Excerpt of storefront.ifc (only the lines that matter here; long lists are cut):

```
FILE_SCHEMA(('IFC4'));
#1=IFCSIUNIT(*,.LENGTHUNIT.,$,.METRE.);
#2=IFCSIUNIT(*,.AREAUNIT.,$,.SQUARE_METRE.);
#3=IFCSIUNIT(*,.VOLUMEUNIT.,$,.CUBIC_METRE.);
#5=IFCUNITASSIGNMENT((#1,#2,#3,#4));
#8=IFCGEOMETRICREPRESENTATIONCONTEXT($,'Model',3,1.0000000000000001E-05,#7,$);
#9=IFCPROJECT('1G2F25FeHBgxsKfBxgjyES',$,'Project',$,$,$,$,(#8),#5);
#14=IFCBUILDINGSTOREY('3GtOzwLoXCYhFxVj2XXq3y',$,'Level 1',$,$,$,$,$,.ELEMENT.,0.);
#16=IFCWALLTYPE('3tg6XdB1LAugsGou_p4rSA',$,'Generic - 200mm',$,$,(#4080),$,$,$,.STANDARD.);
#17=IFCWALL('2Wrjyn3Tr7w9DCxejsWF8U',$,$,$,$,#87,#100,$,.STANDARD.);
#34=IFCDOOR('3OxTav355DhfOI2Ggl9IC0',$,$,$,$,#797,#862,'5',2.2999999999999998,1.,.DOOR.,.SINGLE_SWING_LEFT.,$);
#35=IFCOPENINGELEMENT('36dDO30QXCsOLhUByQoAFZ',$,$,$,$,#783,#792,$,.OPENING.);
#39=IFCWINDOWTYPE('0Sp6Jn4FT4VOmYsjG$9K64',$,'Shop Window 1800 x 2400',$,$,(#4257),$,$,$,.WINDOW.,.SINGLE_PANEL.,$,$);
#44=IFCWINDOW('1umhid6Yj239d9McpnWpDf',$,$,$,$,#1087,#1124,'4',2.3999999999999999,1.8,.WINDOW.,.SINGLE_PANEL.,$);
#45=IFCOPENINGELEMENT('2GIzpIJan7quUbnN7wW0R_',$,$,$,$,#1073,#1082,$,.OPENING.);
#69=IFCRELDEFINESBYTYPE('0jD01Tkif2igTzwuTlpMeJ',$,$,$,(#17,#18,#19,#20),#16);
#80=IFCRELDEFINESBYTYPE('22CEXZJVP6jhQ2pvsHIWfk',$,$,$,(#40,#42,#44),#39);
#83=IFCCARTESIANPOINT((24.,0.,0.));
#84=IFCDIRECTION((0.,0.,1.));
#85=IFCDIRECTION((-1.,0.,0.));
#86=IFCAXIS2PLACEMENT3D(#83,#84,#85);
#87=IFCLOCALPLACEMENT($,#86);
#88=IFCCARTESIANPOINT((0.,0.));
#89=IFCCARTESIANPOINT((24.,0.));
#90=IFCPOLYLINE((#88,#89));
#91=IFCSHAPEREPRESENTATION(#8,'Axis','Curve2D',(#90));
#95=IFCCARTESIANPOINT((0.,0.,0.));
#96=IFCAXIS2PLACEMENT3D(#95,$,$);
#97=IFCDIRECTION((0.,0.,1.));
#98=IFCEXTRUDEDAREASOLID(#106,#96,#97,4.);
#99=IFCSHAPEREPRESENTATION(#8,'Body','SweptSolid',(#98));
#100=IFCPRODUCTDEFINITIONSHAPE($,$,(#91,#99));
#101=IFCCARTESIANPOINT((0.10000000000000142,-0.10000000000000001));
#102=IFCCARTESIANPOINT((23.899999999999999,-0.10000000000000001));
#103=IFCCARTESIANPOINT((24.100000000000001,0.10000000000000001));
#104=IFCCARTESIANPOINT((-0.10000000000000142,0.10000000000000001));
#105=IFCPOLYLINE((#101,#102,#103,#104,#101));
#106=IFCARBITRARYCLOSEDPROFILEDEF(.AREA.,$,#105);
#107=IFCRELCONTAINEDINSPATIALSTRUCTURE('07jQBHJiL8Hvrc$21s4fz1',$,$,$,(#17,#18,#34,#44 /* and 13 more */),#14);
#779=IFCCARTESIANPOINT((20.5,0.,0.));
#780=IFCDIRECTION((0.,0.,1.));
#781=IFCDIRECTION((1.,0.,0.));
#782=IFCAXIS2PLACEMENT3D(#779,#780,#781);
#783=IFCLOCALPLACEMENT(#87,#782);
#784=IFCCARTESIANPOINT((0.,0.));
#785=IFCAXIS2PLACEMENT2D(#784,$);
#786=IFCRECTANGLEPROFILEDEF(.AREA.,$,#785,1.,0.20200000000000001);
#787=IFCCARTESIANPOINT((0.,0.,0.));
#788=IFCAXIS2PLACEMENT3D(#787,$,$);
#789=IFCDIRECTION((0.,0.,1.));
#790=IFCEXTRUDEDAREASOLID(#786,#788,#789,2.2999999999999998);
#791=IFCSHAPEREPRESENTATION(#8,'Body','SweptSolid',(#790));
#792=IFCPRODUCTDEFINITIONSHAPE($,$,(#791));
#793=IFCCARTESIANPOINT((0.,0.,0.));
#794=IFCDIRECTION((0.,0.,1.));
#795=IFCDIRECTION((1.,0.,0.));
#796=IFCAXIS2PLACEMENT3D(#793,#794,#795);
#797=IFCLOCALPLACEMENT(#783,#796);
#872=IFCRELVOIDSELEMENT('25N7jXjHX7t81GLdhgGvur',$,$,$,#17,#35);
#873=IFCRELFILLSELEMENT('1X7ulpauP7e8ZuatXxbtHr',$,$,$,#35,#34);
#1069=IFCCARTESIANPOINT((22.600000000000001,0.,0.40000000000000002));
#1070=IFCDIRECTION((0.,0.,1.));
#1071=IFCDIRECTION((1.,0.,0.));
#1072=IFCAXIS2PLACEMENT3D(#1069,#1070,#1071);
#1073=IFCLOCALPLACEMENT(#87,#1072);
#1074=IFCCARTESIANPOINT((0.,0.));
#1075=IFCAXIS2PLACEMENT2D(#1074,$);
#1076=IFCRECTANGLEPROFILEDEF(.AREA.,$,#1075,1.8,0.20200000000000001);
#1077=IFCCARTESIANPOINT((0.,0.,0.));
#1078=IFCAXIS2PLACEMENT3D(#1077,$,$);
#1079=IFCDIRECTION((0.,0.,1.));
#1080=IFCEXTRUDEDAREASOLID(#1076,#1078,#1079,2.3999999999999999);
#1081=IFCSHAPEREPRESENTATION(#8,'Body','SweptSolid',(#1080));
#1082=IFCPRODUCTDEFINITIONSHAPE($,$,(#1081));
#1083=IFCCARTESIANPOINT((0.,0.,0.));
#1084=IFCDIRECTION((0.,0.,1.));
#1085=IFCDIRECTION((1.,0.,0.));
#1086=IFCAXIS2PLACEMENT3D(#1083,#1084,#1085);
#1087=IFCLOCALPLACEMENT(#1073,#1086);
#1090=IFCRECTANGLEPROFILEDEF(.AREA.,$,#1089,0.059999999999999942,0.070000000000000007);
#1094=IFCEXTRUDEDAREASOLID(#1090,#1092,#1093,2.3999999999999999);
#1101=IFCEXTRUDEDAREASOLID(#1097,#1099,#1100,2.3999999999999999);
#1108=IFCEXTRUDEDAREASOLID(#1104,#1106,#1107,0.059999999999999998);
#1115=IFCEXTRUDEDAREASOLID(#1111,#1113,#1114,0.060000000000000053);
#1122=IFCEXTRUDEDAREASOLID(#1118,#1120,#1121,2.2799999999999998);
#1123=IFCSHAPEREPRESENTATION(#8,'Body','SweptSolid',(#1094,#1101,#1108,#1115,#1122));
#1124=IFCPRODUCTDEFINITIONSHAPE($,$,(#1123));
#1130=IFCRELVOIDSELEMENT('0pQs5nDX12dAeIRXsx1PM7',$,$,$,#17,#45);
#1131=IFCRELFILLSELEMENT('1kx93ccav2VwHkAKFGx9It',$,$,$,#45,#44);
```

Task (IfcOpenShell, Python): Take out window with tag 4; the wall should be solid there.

```python
import ifcopenshell
import ifcopenshell.api.feature
import ifcopenshell.api.root
import ifcopenshell.geom
import ifcopenshell.util.shape

model = ifcopenshell.open("storefront.ifc")
settings = ifcopenshell.geom.settings()


def volume(element):
    """Net volume in cubic metres, openings subtracted."""
    shape = ifcopenshell.geom.create_shape(settings, element)
    return ifcopenshell.util.shape.get_volume(shape.geometry)


window = model.by_guid("1umhid6Yj239d9McpnWpDf")
opening = window.FillsVoids[0].RelatingOpeningElement
wall = opening.VoidsElements[0].RelatingBuildingElement
before = volume(wall)

ifcopenshell.api.root.remove_product(model, product=window)
ifcopenshell.api.feature.remove_feature(model, feature=opening)

after = volume(wall)

print(f"wall volume {before:.3f} -> {after:.3f} m3")

model.write("storefront_updated.ifc")
```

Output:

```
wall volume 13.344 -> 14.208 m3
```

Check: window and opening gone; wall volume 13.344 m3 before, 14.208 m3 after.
